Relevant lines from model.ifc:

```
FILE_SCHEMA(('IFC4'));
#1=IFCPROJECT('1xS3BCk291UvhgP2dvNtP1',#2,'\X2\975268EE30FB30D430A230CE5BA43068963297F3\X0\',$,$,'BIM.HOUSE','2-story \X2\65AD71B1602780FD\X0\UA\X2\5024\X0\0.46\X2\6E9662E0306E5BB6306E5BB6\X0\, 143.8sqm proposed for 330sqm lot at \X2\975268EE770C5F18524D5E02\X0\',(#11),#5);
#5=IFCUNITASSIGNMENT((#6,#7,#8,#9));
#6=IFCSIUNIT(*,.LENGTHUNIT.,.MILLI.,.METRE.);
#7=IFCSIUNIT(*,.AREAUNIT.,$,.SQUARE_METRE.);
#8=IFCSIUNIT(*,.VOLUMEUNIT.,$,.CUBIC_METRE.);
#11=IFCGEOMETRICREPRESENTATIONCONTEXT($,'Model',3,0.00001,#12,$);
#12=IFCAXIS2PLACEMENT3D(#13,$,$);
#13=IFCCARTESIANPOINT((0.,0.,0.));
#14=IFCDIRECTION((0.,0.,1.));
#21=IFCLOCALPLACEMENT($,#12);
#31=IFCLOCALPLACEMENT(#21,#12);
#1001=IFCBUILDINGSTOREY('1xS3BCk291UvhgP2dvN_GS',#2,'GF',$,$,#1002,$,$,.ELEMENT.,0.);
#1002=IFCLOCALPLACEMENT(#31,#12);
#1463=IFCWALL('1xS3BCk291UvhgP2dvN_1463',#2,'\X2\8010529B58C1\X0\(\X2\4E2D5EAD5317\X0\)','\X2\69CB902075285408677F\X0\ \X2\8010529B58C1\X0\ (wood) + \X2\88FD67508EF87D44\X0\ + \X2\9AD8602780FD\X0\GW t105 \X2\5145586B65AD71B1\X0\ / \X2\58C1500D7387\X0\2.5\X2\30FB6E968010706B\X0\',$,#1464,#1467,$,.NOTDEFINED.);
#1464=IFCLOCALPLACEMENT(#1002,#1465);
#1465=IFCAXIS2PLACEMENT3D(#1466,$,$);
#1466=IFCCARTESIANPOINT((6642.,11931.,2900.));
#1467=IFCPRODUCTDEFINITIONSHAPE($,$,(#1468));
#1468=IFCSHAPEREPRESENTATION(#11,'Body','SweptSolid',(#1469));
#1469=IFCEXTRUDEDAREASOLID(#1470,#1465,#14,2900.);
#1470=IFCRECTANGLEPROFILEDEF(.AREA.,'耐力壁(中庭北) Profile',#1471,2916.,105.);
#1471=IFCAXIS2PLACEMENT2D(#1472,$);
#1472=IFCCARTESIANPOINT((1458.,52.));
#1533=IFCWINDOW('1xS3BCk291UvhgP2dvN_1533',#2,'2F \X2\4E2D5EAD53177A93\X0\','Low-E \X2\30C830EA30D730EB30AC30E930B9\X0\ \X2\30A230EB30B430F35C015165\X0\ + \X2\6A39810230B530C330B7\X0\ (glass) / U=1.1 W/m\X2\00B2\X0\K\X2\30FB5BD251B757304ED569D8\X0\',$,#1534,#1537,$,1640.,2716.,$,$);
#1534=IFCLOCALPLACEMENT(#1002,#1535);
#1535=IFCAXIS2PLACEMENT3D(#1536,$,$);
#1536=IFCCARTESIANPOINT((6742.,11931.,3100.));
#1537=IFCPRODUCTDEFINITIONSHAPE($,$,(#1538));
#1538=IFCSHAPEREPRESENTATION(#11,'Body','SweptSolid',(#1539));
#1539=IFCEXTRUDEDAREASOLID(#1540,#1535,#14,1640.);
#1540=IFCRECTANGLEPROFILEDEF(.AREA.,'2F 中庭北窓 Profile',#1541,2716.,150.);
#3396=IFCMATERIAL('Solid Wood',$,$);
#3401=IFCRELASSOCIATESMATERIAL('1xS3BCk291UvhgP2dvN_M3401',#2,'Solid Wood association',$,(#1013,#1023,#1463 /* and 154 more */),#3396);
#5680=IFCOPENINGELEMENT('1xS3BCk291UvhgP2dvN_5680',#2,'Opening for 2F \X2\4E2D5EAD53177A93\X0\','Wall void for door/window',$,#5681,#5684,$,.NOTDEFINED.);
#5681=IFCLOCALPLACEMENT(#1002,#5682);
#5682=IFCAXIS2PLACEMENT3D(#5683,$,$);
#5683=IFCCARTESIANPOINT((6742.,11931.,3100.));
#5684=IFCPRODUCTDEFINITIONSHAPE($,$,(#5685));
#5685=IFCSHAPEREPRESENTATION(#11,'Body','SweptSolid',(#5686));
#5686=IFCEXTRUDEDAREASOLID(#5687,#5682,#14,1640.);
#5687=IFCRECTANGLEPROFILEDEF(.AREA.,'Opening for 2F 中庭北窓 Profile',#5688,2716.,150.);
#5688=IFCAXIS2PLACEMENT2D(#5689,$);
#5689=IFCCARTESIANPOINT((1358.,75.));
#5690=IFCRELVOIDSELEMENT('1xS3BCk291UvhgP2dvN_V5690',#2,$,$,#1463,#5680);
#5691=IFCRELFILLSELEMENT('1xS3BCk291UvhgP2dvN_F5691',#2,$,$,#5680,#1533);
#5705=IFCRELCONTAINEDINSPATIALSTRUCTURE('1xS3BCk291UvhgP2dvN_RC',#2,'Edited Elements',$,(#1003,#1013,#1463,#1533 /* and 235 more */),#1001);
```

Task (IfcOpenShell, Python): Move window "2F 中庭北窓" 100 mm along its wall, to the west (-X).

```python
import ifcopenshell
import ifcopenshell.api.geometry
import ifcopenshell.util.placement
import ifcopenshell.util.unit

model = ifcopenshell.open("model.ifc")
unit_scale = ifcopenshell.util.unit.calculate_unit_scale(model)

window = model.by_id(1533)
opening = window.FillsVoids[0].RelatingOpeningElement
wall = opening.VoidsElements[0].RelatingBuildingElement

wall_matrix = ifcopenshell.util.placement.get_local_placement(wall.ObjectPlacement)
shift = wall_matrix[:3, 0] * -0.1 / unit_scale
before = ifcopenshell.util.placement.get_local_placement(window.ObjectPlacement)[:3, 3].copy()

# The window is not placed relative to its opening, so move both.
for product in (opening, window):
    matrix = ifcopenshell.util.placement.get_local_placement(product.ObjectPlacement)
    matrix[:3, 3] += shift
    ifcopenshell.api.geometry.edit_object_placement(model, product=product, matrix=matrix, is_si=False)

after = ifcopenshell.util.placement.get_local_placement(window.ObjectPlacement)[:3, 3]
print("window moved by", (after - before).round(3) + 0.0)

model.write("model_edited.ifc")
```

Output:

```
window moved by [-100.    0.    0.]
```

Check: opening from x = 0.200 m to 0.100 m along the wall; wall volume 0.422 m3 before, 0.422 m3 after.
